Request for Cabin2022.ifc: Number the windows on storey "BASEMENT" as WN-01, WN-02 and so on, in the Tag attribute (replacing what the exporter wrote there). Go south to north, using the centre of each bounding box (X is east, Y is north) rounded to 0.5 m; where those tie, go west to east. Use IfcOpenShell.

First a look at what the model holds.

```python
import ifcopenshell
import ifcopenshell.util.element
import ifcopenshell.util.placement

model = ifcopenshell.open("Cabin2022.ifc")
print(model.schema)
storey = next(s for s in model.by_type("IfcBuildingStorey") if s.Name == "BASEMENT")
windows = [e for e in ifcopenshell.util.element.get_decomposition(storey) if e.is_a("IfcWindow")]
for e in sorted(windows, key=lambda e: e.id()):
    origin = ifcopenshell.util.placement.get_local_placement(e.ObjectPlacement)[:3, 3]
    print(e.id(), e.Tag, e.Name, origin.round(2) + 0.0, sep=" | ")
```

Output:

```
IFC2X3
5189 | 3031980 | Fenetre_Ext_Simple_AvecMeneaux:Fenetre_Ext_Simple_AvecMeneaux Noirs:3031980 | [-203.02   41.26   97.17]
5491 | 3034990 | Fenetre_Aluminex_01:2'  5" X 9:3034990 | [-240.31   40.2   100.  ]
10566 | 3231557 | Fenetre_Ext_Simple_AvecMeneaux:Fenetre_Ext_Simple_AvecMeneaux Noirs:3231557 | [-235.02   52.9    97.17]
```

```python
import ifcopenshell
import ifcopenshell.geom
import ifcopenshell.util.element
import ifcopenshell.util.shape

model = ifcopenshell.open("Cabin2022.ifc")
settings = ifcopenshell.geom.settings()
settings.set("use-world-coords", True)


def centre(element):
    shape = ifcopenshell.geom.create_shape(settings, element)
    return ifcopenshell.util.shape.get_bbox_centroid(shape.geometry)


storey = next(s for s in model.by_type("IfcBuildingStorey") if s.Name == "BASEMENT")
windows = [e for e in ifcopenshell.util.element.get_decomposition(storey) if e.is_a("IfcWindow")]

# Insertion points can sit at a corner or the storey origin, so sort by the geometry (in metres).
centres = {e: centre(e) for e in windows}
windows.sort(key=lambda e: (round(centres[e][1] / 0.5), centres[e][0]))

for i, e in enumerate(windows, start=1):
    number = f"WN-{i:02d}"
    e.Tag = number
    print(e.id(), number)

model.write("Cabin2022-out.ifc")
```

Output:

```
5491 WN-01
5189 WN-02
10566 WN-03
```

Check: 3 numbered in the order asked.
